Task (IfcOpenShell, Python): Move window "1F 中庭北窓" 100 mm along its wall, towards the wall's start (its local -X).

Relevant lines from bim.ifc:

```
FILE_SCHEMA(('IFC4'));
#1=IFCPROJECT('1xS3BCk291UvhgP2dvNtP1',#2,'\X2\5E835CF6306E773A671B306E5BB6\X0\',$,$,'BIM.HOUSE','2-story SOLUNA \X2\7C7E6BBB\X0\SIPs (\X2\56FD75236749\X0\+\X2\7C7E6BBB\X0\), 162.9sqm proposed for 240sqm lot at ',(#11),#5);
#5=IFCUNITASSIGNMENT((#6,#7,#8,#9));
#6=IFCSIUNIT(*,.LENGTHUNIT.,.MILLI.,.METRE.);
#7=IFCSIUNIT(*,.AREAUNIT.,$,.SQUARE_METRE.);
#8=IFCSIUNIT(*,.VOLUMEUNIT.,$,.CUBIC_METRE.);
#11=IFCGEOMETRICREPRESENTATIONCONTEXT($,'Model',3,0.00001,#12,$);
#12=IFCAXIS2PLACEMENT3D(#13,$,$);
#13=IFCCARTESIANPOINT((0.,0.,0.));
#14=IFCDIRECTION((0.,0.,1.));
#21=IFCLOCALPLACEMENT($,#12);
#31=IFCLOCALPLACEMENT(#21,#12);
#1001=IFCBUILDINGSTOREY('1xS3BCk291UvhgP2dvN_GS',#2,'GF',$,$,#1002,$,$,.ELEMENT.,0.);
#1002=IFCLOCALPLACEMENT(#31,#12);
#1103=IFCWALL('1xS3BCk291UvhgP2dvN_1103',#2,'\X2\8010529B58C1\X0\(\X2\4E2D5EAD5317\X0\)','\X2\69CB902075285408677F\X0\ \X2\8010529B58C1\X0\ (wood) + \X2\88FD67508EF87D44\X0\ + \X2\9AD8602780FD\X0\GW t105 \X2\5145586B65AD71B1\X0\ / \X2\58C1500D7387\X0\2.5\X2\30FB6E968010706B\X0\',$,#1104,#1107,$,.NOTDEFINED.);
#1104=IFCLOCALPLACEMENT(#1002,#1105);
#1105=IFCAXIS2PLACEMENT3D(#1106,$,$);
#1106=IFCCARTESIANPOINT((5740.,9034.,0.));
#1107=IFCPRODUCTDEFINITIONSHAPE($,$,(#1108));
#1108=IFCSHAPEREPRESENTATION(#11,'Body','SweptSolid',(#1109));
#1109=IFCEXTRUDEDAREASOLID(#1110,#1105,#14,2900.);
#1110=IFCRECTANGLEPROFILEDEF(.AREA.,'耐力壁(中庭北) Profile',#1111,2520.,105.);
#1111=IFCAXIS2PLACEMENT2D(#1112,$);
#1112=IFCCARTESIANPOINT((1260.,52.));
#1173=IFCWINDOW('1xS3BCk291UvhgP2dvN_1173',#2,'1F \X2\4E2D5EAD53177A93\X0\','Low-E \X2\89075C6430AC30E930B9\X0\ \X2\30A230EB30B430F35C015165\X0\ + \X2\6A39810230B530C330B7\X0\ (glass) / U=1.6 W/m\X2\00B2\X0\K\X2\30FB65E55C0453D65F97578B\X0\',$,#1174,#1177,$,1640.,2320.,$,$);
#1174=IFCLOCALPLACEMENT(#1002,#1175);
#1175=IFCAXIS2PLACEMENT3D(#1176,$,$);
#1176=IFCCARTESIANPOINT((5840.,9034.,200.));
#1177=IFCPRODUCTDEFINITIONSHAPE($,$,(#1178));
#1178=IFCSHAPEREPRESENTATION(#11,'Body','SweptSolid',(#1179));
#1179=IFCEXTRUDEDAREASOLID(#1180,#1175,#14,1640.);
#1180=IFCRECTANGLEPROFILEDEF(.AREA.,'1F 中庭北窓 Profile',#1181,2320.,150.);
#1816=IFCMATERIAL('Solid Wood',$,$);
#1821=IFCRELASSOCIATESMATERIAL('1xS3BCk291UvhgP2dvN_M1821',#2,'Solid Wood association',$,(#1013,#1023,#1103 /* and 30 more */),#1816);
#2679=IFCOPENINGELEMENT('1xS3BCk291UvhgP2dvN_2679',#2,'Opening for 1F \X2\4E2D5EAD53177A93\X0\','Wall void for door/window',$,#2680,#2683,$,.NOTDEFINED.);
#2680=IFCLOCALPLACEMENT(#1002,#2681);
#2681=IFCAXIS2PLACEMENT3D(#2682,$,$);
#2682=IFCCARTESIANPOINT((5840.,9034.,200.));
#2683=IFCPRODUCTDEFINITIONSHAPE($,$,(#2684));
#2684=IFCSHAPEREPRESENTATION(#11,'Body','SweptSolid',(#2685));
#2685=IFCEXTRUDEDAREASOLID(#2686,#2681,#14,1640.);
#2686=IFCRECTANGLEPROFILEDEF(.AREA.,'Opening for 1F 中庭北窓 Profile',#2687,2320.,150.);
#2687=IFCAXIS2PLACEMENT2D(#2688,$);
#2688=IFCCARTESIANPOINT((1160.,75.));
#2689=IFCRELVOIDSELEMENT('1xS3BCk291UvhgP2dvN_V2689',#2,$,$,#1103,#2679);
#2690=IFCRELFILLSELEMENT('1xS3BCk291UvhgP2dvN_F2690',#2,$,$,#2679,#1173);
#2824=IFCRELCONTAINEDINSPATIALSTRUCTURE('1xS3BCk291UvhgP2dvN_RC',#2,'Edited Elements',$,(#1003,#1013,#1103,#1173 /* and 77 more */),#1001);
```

```python
import ifcopenshell
import ifcopenshell.api.geometry
import ifcopenshell.util.placement
import ifcopenshell.util.unit

model = ifcopenshell.open("bim.ifc")
unit_scale = ifcopenshell.util.unit.calculate_unit_scale(model)

window = model.by_guid("1xS3BCk291UvhgP2dvN_1173")
opening = window.FillsVoids[0].RelatingOpeningElement
wall = opening.VoidsElements[0].RelatingBuildingElement

wall_matrix = ifcopenshell.util.placement.get_local_placement(wall.ObjectPlacement)
shift = wall_matrix[:3, 0] * -0.1 / unit_scale
before = ifcopenshell.util.placement.get_local_placement(window.ObjectPlacement)[:3, 3].copy()

# The window is not placed relative to its opening, so move both.
for product in (opening, window):
    matrix = ifcopenshell.util.placement.get_local_placement(product.ObjectPlacement)
    matrix[:3, 3] += shift
    ifcopenshell.api.geometry.edit_object_placement(model, product=product, matrix=matrix, is_si=False)

after = ifcopenshell.util.placement.get_local_placement(window.ObjectPlacement)[:3, 3]
print("window moved by", (after - before).round(3) + 0.0)

model.write("bim_updated.ifc")
```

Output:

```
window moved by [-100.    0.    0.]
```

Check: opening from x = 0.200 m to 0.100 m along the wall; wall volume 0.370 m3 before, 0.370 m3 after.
